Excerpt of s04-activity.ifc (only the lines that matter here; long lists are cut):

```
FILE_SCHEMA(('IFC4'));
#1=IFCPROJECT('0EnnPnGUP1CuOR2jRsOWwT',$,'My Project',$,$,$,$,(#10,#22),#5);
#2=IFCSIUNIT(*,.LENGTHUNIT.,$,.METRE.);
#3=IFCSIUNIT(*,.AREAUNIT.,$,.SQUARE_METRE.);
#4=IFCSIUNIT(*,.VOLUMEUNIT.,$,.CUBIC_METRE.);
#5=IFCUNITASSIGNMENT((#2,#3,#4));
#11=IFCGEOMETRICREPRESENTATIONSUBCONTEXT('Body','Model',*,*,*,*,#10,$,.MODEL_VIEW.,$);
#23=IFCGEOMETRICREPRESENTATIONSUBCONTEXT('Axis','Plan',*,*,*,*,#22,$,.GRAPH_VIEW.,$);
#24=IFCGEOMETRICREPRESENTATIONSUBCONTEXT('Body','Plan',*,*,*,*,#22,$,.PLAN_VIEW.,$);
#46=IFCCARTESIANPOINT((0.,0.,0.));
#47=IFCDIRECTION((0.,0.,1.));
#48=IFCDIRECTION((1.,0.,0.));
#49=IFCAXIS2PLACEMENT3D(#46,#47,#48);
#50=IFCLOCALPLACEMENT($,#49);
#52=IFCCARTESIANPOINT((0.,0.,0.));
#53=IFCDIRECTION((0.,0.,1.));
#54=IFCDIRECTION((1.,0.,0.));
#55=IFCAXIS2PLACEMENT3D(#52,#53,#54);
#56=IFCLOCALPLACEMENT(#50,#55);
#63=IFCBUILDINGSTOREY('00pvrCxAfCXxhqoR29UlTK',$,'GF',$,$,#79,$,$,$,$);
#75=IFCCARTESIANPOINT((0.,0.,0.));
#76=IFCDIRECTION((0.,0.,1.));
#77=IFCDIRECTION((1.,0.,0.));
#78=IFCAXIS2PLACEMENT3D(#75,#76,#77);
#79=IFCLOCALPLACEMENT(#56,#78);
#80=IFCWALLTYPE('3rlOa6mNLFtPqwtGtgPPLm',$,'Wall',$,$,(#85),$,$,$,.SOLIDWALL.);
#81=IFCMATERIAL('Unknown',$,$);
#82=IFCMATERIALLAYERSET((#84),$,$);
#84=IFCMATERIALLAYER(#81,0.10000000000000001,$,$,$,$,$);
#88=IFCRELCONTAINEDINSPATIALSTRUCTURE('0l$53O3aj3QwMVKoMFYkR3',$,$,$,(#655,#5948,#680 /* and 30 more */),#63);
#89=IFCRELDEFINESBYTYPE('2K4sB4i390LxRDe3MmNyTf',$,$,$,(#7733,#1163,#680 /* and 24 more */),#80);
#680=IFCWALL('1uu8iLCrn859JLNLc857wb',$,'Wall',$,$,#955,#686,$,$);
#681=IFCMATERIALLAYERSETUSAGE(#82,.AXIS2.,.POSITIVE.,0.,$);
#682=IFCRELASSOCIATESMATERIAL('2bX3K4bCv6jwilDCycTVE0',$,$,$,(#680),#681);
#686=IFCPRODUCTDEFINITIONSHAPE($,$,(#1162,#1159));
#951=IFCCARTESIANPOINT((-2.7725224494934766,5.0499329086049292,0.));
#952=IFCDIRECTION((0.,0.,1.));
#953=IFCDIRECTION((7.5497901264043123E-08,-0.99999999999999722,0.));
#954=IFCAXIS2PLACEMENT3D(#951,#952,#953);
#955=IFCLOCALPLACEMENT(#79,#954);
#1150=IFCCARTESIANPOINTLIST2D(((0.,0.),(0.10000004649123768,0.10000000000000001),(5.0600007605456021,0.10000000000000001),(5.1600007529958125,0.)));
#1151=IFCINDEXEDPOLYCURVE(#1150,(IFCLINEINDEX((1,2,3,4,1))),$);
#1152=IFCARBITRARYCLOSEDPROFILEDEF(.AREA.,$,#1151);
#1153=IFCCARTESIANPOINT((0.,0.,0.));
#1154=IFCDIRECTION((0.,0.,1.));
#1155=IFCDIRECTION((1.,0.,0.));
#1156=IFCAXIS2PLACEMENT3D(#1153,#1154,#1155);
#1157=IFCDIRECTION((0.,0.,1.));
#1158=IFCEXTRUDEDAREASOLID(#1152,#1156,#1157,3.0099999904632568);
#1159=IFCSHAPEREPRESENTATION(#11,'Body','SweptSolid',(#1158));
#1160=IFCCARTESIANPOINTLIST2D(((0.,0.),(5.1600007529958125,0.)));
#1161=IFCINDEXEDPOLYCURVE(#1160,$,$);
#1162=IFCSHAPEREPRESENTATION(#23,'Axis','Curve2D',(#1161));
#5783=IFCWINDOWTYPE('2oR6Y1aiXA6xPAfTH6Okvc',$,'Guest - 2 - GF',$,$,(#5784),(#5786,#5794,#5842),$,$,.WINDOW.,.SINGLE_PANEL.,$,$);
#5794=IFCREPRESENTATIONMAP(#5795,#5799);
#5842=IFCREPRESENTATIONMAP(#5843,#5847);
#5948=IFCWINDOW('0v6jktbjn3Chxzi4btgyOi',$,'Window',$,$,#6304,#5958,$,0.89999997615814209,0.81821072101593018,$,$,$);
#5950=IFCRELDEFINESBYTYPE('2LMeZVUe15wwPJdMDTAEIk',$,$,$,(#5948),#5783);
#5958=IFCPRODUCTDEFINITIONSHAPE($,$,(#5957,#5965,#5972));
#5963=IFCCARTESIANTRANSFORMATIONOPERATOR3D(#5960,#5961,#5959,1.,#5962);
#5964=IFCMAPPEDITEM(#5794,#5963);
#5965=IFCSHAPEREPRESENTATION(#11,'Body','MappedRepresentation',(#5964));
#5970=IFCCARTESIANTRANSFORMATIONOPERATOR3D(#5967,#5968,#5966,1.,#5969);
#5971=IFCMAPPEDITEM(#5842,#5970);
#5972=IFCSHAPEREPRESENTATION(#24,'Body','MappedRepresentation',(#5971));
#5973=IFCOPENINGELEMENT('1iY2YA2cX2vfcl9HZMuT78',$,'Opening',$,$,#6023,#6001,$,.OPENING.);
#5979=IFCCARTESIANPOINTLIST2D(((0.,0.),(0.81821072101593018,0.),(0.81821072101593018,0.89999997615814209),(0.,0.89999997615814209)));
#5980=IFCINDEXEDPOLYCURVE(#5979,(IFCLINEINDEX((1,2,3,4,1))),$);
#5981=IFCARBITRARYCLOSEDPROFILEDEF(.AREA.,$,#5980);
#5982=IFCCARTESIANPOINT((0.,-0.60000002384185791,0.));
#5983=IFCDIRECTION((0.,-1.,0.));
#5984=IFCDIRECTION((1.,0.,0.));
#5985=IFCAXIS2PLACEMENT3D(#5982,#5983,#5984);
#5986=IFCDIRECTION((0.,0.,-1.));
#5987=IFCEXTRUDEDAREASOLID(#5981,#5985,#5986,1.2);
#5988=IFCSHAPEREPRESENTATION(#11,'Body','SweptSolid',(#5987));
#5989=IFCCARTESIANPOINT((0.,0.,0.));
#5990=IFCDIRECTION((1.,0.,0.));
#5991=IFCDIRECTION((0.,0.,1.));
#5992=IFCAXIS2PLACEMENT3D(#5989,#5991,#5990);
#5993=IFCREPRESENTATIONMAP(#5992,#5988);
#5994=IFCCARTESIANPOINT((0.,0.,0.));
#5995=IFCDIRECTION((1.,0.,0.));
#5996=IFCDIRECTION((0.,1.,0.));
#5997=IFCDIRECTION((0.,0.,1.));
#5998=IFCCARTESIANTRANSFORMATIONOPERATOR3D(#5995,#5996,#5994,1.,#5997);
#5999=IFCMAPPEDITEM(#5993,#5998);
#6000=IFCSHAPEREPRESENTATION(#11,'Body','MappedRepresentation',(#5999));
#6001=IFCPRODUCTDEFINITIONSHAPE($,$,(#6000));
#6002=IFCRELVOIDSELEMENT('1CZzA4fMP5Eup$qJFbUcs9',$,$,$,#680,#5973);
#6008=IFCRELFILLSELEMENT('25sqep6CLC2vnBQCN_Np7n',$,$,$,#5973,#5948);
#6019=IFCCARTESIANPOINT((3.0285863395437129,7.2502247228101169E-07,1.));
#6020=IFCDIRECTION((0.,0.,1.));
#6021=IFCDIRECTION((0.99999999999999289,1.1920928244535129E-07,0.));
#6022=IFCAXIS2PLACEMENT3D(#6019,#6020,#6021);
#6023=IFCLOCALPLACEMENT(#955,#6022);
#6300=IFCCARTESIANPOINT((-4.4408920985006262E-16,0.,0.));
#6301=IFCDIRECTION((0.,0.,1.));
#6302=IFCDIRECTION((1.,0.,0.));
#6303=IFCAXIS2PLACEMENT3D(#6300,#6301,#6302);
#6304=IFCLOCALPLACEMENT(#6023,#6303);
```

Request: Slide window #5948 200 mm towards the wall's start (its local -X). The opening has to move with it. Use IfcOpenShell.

```python
import ifcopenshell
import ifcopenshell.api.geometry
import ifcopenshell.util.placement
import ifcopenshell.util.unit

model = ifcopenshell.open("s04-activity.ifc")
unit_scale = ifcopenshell.util.unit.calculate_unit_scale(model)

window = model.by_guid("0v6jktbjn3Chxzi4btgyOi")
opening = window.FillsVoids[0].RelatingOpeningElement
wall = opening.VoidsElements[0].RelatingBuildingElement

wall_matrix = ifcopenshell.util.placement.get_local_placement(wall.ObjectPlacement)
shift = wall_matrix[:3, 0] * -0.2 / unit_scale
before = ifcopenshell.util.placement.get_local_placement(window.ObjectPlacement)[:3, 3].copy()

# The window is placed relative to its opening, so it follows when the opening moves.
matrix = ifcopenshell.util.placement.get_local_placement(opening.ObjectPlacement)
matrix[:3, 3] += shift
ifcopenshell.api.geometry.edit_object_placement(
    model, product=opening, matrix=matrix, is_si=False, should_transform_children=True
)

after = ifcopenshell.util.placement.get_local_placement(window.ObjectPlacement)[:3, 3]
print("window moved by", (after - before).round(3) + 0.0)

model.write("s04-activity_rev.ifc")
```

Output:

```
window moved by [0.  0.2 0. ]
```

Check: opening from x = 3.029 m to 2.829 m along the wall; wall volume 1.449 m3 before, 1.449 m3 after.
